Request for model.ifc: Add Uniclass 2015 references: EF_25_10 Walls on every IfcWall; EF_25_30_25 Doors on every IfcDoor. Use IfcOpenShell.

First a look at what the model holds.

```python
import ifcopenshell

model = ifcopenshell.open("model.ifc")
print(model.schema)
print("classifications:", [c.Name for c in model.by_type("IfcClassification")])
for ifc_class in ("IfcDoor", "IfcRoof", "IfcStair", "IfcWall", "IfcWindow"):
    print(ifc_class, len(model.by_type(ifc_class)))
```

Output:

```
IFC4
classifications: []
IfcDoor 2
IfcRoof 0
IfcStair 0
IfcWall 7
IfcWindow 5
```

```python
import ifcopenshell
import ifcopenshell.api.classification

model = ifcopenshell.open("model.ifc")

system = ifcopenshell.api.classification.add_classification(model, classification="Uniclass 2015")

codes = {
    "IfcWall": ("EF_25_10", "Walls"),
    "IfcDoor": ("EF_25_30_25", "Doors"),
}
for ifc_class, (code, name) in codes.items():
    products = model.by_type(ifc_class)
    ifcopenshell.api.classification.add_reference(
        model, products=products, classification=system, identification=code, name=name
    )
    print(code, len(products))

model.write("model_updated.ifc")
```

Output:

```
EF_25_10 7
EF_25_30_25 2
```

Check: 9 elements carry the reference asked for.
